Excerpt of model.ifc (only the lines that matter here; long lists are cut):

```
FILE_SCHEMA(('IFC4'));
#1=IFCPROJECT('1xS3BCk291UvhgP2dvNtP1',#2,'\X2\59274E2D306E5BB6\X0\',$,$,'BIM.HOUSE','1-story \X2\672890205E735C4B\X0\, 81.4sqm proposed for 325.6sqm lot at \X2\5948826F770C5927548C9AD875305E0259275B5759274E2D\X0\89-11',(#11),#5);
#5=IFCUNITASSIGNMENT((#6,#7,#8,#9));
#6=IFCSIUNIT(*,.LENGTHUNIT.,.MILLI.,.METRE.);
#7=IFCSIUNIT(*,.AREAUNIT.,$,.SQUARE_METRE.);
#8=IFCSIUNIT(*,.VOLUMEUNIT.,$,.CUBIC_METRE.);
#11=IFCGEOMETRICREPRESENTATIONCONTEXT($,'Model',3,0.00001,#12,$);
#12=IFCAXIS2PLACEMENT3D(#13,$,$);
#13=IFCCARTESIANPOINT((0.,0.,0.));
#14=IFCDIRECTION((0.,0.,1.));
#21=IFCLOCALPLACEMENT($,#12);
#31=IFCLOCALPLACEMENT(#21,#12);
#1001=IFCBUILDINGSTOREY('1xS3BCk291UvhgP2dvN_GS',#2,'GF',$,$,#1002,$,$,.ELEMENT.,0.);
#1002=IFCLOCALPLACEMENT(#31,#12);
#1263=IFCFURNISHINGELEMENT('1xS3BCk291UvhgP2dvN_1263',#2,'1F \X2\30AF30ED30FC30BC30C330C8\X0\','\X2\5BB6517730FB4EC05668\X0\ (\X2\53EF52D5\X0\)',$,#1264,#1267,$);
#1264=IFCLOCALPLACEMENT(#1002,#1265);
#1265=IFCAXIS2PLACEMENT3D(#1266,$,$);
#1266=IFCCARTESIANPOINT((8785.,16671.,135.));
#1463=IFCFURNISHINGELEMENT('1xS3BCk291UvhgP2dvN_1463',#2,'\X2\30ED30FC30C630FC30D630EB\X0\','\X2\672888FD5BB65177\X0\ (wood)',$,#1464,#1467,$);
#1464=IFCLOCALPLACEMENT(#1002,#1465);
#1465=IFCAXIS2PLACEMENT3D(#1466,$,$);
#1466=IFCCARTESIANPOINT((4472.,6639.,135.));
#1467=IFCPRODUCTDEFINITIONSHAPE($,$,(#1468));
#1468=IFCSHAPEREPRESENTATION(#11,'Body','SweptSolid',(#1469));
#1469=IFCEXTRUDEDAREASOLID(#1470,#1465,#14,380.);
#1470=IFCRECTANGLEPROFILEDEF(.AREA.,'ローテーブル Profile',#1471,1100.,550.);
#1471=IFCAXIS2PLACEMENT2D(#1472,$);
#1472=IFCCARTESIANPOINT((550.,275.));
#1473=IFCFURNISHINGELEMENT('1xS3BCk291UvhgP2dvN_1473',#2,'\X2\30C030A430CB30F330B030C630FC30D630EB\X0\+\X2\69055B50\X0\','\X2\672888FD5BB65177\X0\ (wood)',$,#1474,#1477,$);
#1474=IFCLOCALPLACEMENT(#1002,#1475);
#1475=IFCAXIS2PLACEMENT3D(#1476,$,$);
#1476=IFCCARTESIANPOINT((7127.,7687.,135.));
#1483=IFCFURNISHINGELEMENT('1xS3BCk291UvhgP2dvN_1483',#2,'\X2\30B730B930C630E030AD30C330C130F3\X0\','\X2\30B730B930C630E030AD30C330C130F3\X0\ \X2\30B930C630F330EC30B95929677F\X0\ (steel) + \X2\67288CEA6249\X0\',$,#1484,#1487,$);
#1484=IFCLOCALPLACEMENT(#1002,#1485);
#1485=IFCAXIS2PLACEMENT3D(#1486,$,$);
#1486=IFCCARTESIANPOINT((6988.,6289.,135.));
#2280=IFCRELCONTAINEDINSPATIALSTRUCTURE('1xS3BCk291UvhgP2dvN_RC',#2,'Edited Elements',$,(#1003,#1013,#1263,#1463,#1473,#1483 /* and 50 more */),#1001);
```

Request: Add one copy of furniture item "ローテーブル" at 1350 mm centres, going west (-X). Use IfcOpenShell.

```python
import numpy as np
import ifcopenshell
import ifcopenshell.api.geometry
import ifcopenshell.api.root
import ifcopenshell.util.element
import ifcopenshell.util.placement

model = ifcopenshell.open("model.ifc")


def reuse_history(source, copy):
    """copy_class also copies each property set's owner history, people and application; keep the originals."""
    for rel in copy.IsDefinedBy:
        if rel.is_a("IfcRelDefinesByProperties") and (history := rel.RelatingPropertyDefinition.OwnerHistory):
            rel.RelatingPropertyDefinition.OwnerHistory = source.OwnerHistory
            ifcopenshell.util.element.remove_deep2(model, history)


source = model.by_guid("1xS3BCk291UvhgP2dvN_1463")
base = ifcopenshell.util.placement.get_local_placement(source.ObjectPlacement)
step = np.array([-1.0, 0.0, 0.0]) * 1350.0

for i in range(1, 2):
    copy = ifcopenshell.api.root.copy_class(model, product=source)
    copy.Representation = ifcopenshell.util.element.copy_deep(
        model, source.Representation, exclude=["IfcGeometricRepresentationContext", "IfcRepresentationMap"]
    )
    reuse_history(source, copy)
    matrix = base.copy()
    matrix[:3, 3] += i * step
    print("added at", matrix[:3, 3].round(3) + 0.0)
    ifcopenshell.api.geometry.edit_object_placement(model, product=copy, matrix=matrix, is_si=False)

model.write("model-out.ifc")
```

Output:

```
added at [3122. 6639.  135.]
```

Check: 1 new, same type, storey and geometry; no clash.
